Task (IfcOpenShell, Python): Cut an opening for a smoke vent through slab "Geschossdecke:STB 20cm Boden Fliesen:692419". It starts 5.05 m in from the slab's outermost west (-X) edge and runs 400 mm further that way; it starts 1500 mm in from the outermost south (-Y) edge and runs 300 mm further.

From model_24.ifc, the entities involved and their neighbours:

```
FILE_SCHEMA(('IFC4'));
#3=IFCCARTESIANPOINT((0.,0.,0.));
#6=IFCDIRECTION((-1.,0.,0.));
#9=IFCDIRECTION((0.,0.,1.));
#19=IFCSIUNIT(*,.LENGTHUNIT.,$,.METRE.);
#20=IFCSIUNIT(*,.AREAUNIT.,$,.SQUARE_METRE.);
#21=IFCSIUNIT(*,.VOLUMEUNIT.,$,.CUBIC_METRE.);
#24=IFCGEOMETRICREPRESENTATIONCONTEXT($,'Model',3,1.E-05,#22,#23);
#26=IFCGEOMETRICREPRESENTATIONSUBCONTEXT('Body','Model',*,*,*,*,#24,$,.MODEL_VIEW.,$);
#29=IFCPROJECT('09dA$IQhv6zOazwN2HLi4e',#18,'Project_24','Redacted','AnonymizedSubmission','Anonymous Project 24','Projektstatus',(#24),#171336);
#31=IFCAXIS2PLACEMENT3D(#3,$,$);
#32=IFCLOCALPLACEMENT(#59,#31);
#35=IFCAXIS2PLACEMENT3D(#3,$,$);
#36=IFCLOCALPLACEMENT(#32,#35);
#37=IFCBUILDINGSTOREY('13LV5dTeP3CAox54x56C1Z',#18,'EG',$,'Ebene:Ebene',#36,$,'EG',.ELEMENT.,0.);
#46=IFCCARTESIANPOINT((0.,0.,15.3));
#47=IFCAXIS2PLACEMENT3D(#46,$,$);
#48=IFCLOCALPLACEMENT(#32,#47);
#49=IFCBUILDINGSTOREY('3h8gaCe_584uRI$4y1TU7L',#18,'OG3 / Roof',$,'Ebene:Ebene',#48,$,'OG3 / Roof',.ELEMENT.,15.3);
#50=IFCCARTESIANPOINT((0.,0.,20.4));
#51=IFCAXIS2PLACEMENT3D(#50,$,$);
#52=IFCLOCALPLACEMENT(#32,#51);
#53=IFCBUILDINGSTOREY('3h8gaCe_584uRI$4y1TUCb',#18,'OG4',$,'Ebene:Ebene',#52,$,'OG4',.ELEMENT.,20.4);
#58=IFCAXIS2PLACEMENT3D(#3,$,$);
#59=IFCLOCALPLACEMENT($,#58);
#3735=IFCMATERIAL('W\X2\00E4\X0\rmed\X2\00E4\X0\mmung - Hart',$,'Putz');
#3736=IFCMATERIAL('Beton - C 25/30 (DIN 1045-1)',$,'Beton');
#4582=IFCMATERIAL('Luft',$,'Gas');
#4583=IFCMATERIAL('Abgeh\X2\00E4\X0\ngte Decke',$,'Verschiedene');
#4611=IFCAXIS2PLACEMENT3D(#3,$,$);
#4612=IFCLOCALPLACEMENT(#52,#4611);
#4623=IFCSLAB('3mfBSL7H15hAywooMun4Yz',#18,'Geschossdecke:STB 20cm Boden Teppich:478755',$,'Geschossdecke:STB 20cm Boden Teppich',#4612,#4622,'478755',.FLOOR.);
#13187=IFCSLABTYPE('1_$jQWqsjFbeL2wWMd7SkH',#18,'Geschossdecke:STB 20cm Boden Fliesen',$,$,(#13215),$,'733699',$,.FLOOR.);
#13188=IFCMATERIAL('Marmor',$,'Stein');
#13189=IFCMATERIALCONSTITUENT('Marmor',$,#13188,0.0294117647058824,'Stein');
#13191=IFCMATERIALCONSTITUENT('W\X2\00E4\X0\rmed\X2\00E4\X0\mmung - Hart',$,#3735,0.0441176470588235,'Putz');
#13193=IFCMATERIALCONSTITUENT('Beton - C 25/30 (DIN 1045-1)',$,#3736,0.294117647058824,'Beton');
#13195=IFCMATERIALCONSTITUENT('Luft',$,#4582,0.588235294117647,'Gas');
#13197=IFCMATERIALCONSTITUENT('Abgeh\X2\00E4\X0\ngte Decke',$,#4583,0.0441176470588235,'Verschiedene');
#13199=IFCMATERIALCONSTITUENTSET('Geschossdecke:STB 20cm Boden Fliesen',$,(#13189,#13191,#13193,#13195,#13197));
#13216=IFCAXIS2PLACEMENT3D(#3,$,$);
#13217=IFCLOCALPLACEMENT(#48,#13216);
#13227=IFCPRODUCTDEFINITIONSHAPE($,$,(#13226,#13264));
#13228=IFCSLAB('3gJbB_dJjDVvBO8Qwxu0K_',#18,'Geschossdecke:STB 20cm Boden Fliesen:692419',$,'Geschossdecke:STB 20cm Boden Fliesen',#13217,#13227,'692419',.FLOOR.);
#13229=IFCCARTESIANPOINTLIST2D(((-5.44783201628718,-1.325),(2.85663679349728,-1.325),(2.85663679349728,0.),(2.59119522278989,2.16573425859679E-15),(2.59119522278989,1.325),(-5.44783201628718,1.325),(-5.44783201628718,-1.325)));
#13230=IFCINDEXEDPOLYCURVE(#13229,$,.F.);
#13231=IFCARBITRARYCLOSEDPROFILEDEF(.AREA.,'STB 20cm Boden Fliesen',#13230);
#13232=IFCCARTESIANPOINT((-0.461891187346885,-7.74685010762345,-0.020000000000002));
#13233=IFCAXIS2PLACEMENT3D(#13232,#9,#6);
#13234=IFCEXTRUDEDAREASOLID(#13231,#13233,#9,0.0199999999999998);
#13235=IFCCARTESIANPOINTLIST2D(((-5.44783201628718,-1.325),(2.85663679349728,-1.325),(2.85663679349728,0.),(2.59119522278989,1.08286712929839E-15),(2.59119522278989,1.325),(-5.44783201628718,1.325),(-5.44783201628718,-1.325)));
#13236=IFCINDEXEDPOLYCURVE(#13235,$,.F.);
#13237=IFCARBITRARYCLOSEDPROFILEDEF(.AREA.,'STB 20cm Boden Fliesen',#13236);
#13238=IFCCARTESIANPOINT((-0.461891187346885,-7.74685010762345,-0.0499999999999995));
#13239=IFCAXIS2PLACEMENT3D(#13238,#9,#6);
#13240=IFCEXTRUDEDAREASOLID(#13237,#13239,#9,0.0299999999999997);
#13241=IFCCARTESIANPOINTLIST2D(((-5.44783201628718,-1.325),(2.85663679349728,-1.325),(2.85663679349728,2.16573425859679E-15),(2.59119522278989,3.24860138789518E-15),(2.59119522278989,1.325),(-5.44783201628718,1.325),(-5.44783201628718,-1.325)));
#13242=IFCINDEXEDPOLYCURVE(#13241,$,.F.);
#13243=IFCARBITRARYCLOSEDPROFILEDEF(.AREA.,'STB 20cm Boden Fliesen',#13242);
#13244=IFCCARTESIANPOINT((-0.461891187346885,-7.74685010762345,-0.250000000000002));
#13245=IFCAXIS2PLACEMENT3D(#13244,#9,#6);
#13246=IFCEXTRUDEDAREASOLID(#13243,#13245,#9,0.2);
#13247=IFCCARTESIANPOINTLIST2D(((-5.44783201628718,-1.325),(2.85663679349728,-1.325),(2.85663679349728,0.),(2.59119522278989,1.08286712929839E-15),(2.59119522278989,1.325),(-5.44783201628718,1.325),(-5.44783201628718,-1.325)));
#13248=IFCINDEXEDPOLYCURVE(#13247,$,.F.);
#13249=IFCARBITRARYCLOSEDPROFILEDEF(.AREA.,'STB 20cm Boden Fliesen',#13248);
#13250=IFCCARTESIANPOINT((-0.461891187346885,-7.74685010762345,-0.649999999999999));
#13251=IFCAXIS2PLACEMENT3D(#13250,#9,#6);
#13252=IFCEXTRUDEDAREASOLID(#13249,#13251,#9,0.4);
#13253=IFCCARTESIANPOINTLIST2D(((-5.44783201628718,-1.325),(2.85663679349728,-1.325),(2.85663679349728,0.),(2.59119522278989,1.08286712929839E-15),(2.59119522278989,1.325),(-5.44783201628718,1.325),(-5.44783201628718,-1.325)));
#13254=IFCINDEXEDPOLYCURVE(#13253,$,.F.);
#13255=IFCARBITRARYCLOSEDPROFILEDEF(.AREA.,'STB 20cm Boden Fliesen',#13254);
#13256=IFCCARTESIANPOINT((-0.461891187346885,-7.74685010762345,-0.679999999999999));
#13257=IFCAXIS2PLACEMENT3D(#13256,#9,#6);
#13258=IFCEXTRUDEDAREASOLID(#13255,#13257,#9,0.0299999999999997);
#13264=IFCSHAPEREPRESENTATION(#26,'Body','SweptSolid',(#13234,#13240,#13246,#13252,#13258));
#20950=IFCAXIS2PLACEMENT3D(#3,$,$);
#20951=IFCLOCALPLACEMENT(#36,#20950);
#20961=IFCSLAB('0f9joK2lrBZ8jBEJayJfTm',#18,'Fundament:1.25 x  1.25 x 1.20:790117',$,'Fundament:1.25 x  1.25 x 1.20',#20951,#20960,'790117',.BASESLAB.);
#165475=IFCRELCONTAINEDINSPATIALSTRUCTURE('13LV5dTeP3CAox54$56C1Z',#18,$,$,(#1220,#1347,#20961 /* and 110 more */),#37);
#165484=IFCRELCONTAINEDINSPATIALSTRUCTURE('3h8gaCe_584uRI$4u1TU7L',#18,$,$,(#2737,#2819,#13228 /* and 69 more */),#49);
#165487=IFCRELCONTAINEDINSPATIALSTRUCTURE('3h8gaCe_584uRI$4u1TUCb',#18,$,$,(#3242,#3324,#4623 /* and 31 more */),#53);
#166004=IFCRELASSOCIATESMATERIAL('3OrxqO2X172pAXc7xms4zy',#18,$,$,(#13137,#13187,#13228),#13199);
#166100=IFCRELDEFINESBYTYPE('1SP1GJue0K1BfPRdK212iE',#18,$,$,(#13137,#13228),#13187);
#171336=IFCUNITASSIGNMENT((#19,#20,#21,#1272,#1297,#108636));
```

```python
import numpy as np
import ifcopenshell
import ifcopenshell.api.feature
import ifcopenshell.api.geometry
import ifcopenshell.api.root
import ifcopenshell.geom
import ifcopenshell.util.placement
import ifcopenshell.util.representation
import ifcopenshell.util.shape
import ifcopenshell.util.unit

model = ifcopenshell.open("model_24.ifc")
unit_scale = ifcopenshell.util.unit.calculate_unit_scale(model)
settings = ifcopenshell.geom.settings()


def volume(element):
    """Net volume in cubic metres, openings subtracted."""
    shape = ifcopenshell.geom.create_shape(settings, element)
    return ifcopenshell.util.shape.get_volume(shape.geometry)


slab = model.by_guid("3gJbB_dJjDVvBO8Qwxu0K_")
before = volume(slab)

# Extent in the slab's own axes, in metres. The edges named are its -X and -Y sides.
slab_shape = ifcopenshell.geom.create_shape(settings, slab)
vertices = ifcopenshell.util.shape.get_vertices(slab_shape.geometry)
x_min, y_min, bottom = vertices.min(axis=0)
top = vertices[:, 2].max()

opening = ifcopenshell.api.root.create_entity(model, ifc_class="IfcOpeningElement", name="Smoke vent opening", predefined_type="OPENING")
context = ifcopenshell.util.representation.get_context(model, "Model", "Body", "MODEL_VIEW")
width, depth = 0.4, 0.3
outline = [(0.0, 0.0), (width, 0.0), (width, depth), (0.0, depth), (0.0, 0.0)]
# Overshoot both faces by 50 mm so the cut is clean.
shape = ifcopenshell.api.geometry.add_slab_representation(
    model, context=context, depth=top - bottom + 0.1, polyline=outline
)
ifcopenshell.api.geometry.assign_representation(model, product=opening, representation=shape)

matrix = ifcopenshell.util.placement.get_local_placement(slab.ObjectPlacement)
matrix[:, 3] = matrix @ np.append(np.array([x_min + 5.05, y_min + 1.5, bottom - 0.05]) / unit_scale, 1.0)
ifcopenshell.api.geometry.edit_object_placement(model, product=opening, matrix=matrix, is_si=False)
ifcopenshell.api.feature.add_feature(model, feature=opening, element=slab)

after = volume(slab)

print(f"slab volume {before:.3f} -> {after:.3f} m3")

model.write("model_24_v2.ifc")
```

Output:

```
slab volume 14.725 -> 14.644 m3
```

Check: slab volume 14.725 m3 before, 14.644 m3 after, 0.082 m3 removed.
